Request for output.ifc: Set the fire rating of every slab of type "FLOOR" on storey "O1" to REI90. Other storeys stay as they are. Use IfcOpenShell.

First a look at what the model holds.

```python
import ifcopenshell
import ifcopenshell.util.element

model = ifcopenshell.open("output.ifc")
print(model.schema)
storey = next(s for s in model.by_type("IfcBuildingStorey") if s.Name == "O1")
slabs = [e for e in ifcopenshell.util.element.get_decomposition(storey) if e.is_a("IfcSlab")]
seen = {}
for e in slabs:
    element_type = ifcopenshell.util.element.get_type(e)
    key = (element_type.Name if element_type != e and element_type else None, ifcopenshell.util.element.get_pset(e, "Pset_SlabCommon", "FireRating"))
    seen[key] = seen.get(key, 0) + 1
for (name, value), count in sorted(seen.items(), key=str):
    print(count, "x", name, "|", value)
```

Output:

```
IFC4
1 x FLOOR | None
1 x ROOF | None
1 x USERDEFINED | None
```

```python
import ifcopenshell
import ifcopenshell.api.pset
import ifcopenshell.util.element

model = ifcopenshell.open("output.ifc")

storey = next(s for s in model.by_type("IfcBuildingStorey") if s.Name == "O1")
slabs = [e for e in ifcopenshell.util.element.get_decomposition(storey) if e.is_a("IfcSlab")]

count = 0
for e in slabs:
    element_type = ifcopenshell.util.element.get_type(e)
    if element_type in (None, e) or element_type.Name != "FLOOR":
        continue
    # add_pset returns the element's existing set when there is one.
    pset = ifcopenshell.api.pset.add_pset(model, product=e, name="Pset_SlabCommon")
    ifcopenshell.api.pset.edit_pset(model, pset=pset, properties={"FireRating": "REI90"})
    count += 1

print(count, "slabs updated")

model.write("output_v2.ifc")
```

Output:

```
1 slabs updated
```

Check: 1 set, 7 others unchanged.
